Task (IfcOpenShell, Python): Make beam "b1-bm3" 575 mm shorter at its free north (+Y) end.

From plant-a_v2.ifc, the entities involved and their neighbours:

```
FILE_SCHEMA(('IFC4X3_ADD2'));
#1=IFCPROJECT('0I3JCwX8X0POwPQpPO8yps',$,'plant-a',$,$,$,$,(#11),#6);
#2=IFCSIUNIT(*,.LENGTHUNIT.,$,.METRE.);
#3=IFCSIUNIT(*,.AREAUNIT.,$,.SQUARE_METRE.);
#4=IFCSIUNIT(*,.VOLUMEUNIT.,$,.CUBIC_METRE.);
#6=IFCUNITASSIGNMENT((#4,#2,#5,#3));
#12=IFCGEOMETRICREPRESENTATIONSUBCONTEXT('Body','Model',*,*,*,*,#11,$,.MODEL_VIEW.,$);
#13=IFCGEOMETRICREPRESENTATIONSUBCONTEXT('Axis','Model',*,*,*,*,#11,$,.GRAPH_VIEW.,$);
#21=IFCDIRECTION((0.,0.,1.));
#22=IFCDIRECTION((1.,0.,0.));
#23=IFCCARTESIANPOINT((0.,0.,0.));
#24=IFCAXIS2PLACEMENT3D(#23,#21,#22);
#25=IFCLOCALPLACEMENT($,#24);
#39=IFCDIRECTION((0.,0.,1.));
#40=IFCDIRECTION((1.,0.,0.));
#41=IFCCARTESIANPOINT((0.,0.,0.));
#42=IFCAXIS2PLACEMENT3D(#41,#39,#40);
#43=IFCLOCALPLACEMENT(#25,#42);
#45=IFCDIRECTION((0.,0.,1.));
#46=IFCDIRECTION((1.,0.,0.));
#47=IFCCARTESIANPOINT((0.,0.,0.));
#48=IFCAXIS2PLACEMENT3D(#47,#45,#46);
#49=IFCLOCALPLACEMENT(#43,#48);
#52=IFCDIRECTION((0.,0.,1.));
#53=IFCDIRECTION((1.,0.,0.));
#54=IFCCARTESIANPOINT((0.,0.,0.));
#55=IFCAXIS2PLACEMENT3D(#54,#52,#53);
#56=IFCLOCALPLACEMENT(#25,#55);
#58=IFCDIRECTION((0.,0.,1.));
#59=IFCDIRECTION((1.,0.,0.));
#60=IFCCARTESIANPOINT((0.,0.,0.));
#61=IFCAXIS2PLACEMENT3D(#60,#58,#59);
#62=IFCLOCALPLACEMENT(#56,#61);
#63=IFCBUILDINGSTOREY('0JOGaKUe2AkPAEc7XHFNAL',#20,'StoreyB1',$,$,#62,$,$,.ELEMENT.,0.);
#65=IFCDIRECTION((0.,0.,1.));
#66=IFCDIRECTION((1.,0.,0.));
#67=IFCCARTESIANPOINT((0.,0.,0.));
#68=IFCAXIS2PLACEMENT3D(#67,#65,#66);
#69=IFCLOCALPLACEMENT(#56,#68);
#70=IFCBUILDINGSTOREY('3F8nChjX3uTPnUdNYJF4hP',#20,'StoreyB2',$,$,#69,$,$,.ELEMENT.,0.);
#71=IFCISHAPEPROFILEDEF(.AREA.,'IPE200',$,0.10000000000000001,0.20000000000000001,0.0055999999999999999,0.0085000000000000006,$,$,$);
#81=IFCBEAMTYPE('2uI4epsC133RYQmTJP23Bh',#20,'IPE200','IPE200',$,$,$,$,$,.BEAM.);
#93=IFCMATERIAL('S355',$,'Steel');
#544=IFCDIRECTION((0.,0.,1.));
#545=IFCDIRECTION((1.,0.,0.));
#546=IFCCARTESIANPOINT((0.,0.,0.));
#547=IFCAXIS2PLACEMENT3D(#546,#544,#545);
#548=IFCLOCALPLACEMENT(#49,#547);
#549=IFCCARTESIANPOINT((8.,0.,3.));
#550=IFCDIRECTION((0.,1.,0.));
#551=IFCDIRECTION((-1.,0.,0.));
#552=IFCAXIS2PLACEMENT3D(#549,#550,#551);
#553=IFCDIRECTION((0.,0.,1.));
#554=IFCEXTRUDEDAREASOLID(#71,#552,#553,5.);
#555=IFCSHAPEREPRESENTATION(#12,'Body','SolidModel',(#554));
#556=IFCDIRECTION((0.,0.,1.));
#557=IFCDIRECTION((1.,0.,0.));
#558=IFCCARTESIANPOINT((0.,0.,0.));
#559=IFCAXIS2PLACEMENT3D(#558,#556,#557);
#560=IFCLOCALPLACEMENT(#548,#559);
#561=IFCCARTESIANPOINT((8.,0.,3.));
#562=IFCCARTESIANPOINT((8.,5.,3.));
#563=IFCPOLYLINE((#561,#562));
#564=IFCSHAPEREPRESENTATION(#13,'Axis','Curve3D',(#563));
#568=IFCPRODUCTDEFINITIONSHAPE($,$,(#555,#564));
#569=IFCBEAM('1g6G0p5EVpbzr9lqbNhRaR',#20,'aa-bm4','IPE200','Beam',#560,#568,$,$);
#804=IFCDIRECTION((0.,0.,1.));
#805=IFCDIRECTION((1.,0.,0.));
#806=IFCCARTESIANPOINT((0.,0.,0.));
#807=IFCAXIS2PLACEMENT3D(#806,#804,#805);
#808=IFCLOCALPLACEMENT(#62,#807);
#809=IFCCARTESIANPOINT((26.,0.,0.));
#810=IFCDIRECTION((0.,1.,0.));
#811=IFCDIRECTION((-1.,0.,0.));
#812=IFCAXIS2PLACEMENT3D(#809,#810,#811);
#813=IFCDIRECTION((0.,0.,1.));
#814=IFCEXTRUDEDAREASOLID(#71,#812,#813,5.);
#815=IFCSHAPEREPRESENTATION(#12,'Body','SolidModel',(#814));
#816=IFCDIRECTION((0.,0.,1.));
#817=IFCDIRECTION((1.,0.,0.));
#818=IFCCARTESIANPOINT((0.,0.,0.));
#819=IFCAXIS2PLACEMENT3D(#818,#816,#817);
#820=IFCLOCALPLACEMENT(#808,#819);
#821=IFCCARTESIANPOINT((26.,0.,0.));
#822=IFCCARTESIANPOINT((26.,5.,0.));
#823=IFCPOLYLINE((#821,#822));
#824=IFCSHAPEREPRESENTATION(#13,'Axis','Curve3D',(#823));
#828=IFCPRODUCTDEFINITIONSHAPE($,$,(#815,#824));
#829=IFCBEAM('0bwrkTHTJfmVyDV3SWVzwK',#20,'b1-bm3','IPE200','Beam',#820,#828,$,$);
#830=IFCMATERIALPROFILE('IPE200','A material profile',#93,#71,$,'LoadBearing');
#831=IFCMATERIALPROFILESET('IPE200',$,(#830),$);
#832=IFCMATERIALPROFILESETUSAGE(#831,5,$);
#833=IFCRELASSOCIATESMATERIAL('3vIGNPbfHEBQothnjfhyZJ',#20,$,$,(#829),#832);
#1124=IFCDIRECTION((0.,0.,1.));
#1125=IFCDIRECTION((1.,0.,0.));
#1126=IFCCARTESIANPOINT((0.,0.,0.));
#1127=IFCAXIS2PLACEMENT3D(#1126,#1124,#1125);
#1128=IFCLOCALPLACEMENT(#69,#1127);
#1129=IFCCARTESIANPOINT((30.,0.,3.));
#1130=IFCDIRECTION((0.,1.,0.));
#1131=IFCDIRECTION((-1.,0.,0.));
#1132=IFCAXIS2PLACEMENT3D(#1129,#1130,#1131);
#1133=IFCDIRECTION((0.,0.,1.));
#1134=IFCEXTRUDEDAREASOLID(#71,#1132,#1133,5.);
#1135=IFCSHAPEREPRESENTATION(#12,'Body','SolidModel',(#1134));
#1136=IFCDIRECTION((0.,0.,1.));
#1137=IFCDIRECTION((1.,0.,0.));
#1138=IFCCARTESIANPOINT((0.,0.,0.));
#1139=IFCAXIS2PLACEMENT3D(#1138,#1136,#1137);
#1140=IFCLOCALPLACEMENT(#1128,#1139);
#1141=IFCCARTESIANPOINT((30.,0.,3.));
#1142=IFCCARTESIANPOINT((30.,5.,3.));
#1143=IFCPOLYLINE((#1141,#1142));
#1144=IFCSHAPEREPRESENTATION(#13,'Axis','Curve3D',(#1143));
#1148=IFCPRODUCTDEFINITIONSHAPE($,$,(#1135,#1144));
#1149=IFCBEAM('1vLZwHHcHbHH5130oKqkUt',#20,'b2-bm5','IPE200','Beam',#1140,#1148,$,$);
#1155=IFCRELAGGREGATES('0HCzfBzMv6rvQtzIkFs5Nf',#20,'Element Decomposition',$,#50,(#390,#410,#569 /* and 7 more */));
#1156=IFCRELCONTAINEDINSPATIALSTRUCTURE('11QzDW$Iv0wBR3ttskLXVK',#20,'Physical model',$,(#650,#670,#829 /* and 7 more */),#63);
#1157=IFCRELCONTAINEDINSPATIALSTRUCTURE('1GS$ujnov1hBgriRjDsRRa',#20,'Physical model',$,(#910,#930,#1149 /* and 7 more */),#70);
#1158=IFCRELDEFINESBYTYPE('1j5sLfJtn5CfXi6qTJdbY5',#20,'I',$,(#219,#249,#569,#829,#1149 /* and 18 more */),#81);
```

```python
import numpy as np
import ifcopenshell
import ifcopenshell.util.representation
import ifcopenshell.util.unit

model = ifcopenshell.open("plant-a_v2.ifc")
unit_scale = ifcopenshell.util.unit.calculate_unit_scale(model)

member = model.by_guid("0bwrkTHTJfmVyDV3SWVzwK")
change = -0.575 / unit_scale

# The extrusion runs towards the end named, so only its depth changes.
body = ifcopenshell.util.representation.get_representation(member, "Model", "Body")
solid = body.Items[0]
old_length = solid.Depth
solid.Depth += change

# Move the axis end point with it.
axis = next(r for r in member.Representation.Representations if r.RepresentationIdentifier == "Axis").Items[0]
start, end = (np.array(p.Coordinates) for p in axis.Points)
end = end + (end - start) / np.linalg.norm(end - start) * change
point = model.createIfcCartesianPoint(end.tolist())
axis.Points = [axis.Points[0], point]

print(f"length {old_length:g} -> {solid.Depth:g}")

model.write("plant-a_v2_updated.ifc")
```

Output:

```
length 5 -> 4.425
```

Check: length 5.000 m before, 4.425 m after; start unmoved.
